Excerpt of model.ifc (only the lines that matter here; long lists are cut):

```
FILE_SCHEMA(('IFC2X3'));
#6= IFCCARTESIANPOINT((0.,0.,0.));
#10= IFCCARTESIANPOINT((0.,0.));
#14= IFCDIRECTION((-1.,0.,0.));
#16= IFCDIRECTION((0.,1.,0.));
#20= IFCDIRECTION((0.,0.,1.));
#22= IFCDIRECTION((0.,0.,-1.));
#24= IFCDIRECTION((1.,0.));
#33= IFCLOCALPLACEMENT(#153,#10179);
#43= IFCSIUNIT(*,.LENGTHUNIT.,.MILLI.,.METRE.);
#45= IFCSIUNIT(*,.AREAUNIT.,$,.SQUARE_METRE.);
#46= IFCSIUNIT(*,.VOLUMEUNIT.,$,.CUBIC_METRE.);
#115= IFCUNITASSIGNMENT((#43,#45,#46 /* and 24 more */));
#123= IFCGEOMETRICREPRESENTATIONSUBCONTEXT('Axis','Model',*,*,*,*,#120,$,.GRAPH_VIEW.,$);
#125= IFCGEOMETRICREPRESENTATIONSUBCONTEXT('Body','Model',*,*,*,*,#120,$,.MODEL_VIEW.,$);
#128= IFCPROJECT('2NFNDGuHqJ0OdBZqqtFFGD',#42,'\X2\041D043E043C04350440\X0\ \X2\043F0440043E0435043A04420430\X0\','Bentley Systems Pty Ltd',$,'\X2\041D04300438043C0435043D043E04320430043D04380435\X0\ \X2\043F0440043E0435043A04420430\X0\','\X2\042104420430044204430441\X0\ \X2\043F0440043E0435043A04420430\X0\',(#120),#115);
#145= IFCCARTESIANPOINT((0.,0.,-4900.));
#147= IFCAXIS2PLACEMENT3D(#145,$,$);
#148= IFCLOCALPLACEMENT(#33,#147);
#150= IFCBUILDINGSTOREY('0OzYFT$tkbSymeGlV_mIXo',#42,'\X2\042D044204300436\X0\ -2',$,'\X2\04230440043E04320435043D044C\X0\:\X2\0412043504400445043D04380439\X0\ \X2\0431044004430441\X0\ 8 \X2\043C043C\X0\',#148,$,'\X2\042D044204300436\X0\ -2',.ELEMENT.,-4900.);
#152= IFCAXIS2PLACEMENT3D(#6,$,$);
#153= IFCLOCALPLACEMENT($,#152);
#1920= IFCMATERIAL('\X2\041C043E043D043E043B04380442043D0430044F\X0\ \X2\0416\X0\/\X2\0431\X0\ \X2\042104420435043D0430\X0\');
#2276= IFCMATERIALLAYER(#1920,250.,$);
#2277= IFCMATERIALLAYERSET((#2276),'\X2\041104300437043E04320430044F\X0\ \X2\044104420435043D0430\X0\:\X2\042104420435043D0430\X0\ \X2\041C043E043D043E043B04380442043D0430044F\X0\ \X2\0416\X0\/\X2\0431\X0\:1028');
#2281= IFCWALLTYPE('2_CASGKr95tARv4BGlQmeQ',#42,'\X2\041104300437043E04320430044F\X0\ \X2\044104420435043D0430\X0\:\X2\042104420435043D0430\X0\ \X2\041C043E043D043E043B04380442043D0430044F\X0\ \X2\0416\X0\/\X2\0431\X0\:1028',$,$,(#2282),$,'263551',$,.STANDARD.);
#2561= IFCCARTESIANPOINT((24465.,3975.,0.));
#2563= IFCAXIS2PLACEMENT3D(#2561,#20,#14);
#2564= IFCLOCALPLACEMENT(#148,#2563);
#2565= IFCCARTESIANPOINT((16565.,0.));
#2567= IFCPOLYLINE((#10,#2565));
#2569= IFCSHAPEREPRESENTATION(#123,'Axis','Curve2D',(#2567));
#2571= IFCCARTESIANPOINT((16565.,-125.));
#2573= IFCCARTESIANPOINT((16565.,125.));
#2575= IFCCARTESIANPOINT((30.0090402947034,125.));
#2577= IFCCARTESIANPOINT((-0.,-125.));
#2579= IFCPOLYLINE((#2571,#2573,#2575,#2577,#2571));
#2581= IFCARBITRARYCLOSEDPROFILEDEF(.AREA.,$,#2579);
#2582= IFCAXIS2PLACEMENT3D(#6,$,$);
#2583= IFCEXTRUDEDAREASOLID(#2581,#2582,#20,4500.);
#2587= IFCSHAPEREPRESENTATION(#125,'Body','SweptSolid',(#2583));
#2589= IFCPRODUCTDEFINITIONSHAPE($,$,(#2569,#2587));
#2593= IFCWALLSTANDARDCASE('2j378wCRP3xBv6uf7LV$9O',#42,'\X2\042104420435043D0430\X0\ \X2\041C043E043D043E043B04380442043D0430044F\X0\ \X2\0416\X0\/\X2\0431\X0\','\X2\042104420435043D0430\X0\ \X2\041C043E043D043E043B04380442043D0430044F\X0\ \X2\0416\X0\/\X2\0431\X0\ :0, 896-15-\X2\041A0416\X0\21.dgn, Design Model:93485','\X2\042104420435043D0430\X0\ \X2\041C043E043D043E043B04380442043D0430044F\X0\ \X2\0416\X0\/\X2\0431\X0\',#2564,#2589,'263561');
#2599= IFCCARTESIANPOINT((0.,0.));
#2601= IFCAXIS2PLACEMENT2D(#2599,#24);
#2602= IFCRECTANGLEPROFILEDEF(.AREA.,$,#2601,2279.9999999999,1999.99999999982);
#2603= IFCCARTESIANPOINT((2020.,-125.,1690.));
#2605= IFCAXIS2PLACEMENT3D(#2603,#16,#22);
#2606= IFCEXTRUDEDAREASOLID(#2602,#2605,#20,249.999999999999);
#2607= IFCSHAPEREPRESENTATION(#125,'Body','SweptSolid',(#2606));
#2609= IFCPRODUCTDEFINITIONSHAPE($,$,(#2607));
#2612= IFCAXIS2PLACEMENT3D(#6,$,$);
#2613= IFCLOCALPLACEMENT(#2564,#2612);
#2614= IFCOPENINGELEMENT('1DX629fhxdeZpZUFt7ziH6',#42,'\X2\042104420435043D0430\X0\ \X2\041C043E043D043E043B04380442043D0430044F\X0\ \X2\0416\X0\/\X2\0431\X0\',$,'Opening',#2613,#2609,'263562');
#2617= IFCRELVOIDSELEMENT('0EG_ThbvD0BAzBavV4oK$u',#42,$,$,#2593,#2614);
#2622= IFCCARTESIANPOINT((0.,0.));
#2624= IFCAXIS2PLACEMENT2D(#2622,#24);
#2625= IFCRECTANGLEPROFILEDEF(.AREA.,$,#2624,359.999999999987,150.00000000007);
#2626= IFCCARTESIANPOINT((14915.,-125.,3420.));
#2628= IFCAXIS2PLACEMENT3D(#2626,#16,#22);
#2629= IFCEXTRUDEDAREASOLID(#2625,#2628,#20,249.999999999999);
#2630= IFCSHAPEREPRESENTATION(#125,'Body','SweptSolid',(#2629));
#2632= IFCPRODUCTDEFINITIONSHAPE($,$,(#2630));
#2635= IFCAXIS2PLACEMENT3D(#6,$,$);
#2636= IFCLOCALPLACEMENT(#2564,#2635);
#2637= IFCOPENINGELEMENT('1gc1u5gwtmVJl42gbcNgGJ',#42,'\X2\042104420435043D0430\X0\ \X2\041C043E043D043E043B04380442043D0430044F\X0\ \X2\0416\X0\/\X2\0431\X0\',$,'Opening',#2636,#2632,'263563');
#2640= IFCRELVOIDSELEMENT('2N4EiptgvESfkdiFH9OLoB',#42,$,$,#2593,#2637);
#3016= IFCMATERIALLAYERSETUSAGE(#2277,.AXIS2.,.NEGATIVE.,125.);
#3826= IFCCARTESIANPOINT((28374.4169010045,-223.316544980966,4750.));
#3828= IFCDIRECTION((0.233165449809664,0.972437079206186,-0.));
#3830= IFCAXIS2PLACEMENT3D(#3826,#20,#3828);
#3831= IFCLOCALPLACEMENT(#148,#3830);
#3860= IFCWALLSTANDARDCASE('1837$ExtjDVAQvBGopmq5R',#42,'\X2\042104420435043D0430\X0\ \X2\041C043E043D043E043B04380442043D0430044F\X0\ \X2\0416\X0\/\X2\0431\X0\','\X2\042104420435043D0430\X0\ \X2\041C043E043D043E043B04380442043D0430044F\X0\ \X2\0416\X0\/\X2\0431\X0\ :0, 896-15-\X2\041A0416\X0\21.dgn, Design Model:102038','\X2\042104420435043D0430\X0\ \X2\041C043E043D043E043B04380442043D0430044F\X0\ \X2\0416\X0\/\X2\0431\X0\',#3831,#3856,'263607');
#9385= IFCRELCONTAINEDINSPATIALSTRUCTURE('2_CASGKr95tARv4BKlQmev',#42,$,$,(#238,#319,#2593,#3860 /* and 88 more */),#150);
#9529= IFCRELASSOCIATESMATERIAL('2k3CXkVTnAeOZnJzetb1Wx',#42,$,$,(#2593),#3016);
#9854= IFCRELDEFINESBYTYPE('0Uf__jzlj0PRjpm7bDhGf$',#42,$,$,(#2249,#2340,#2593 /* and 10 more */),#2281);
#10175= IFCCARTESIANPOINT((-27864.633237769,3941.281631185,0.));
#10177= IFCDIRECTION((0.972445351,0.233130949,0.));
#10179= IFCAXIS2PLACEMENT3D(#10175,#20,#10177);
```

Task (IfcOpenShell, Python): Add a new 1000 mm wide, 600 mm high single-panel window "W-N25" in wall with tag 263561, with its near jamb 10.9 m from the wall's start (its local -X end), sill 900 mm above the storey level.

```python
import numpy as np
import ifcopenshell
import ifcopenshell.api.feature
import ifcopenshell.api.geometry
import ifcopenshell.api.root
import ifcopenshell.api.spatial
import ifcopenshell.api.type
import ifcopenshell.geom
import ifcopenshell.util.element
import ifcopenshell.util.placement
import ifcopenshell.util.representation
import ifcopenshell.util.shape
import ifcopenshell.util.unit

model = ifcopenshell.open("model.ifc")
unit_scale = ifcopenshell.util.unit.calculate_unit_scale(model)
settings = ifcopenshell.geom.settings()


def volume(element):
    """Net volume in cubic metres, openings subtracted."""
    shape = ifcopenshell.geom.create_shape(settings, element)
    return ifcopenshell.util.shape.get_volume(shape.geometry)


wall = model.by_guid("2j378wCRP3xBv6uf7LV$9O")
storey = ifcopenshell.util.element.get_container(wall, ifc_class="IfcBuildingStorey")
context = ifcopenshell.util.representation.get_context(model, "Model", "Body", "MODEL_VIEW")
before = volume(wall)

width, height, from_end, sill = 1, 0.6, 10.9, 0.9  # metres

# The wall runs along its own X axis, and the end named is its -X end.
wall_shape = ifcopenshell.geom.create_shape(settings, wall)
x, y, z = ifcopenshell.util.shape.get_vertices(wall_shape.geometry).T
start = x.min() + from_end
face, thickness = float(y.min()), float(y.max() - y.min())
wall_matrix = ifcopenshell.util.placement.get_local_placement(wall.ObjectPlacement)
level = ifcopenshell.util.placement.get_local_placement(storey.ObjectPlacement)[2, 3]


def in_wall(x, y):
    """Placement at x, y metres in the wall's axes, at sill height."""
    matrix = wall_matrix.copy()
    matrix[:, 3] = wall_matrix @ np.array([x / unit_scale, y / unit_scale, 0.0, 1.0])
    matrix[2, 3] = level + sill / unit_scale
    return matrix


# Opening: a box that overshoots both wall faces by 50 mm.
opening = ifcopenshell.api.root.create_entity(model, ifc_class="IfcOpeningElement")
box = ifcopenshell.api.geometry.add_wall_representation(
    model, context=context, length=width, height=height, thickness=thickness + 0.1
)
ifcopenshell.api.geometry.assign_representation(model, product=opening, representation=box)
ifcopenshell.api.geometry.edit_object_placement(model, product=opening, matrix=in_wall(start, face - 0.05), is_si=False)
ifcopenshell.api.feature.add_feature(model, feature=opening, element=wall)

window = ifcopenshell.api.root.create_entity(model, ifc_class="IfcWindow", name="W-N25")
window.OverallWidth, window.OverallHeight = width / unit_scale, height / unit_scale
body = ifcopenshell.api.geometry.add_window_representation(
    model,
    context=context,
    overall_width=window.OverallWidth,
    overall_height=window.OverallHeight,
    partition_type="SINGLE_PANEL",
)
ifcopenshell.api.geometry.assign_representation(model, product=window, representation=body)
ifcopenshell.api.spatial.assign_container(model, products=[window], relating_structure=storey)
fills = ifcopenshell.api.feature.add_filling(model, opening=opening, element=window)
fills.OwnerHistory = window.OwnerHistory  # required in IFC2X3

# IFC2X3 keeps the operation on the window style.
style = ifcopenshell.api.root.create_entity(model, ifc_class="IfcWindowStyle", name="W-N25")
style.OperationType, style.ConstructionType = "SINGLE_PANEL", "NOTDEFINED"
style.ParameterTakesPrecedence = style.Sizeable = False
ifcopenshell.api.type.assign_type(model, related_objects=[window], relating_type=style)

# Centre the window in the wall's thickness.
ifcopenshell.api.geometry.edit_object_placement(model, product=window, matrix=in_wall(start, face), is_si=False)
window_shape = ifcopenshell.geom.create_shape(settings, window)
depth = ifcopenshell.util.shape.get_vertices(window_shape.geometry)[:, 1]
offset = face + thickness / 2 - (depth.min() + depth.max()) / 2
ifcopenshell.api.geometry.edit_object_placement(model, product=window, matrix=in_wall(start, offset), is_si=False)

after = volume(wall)

print(f"wall volume {before:.3f} -> {after:.3f} m3")

model.write("model_updated.ifc")
```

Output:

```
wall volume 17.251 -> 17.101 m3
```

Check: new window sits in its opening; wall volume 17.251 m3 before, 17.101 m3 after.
